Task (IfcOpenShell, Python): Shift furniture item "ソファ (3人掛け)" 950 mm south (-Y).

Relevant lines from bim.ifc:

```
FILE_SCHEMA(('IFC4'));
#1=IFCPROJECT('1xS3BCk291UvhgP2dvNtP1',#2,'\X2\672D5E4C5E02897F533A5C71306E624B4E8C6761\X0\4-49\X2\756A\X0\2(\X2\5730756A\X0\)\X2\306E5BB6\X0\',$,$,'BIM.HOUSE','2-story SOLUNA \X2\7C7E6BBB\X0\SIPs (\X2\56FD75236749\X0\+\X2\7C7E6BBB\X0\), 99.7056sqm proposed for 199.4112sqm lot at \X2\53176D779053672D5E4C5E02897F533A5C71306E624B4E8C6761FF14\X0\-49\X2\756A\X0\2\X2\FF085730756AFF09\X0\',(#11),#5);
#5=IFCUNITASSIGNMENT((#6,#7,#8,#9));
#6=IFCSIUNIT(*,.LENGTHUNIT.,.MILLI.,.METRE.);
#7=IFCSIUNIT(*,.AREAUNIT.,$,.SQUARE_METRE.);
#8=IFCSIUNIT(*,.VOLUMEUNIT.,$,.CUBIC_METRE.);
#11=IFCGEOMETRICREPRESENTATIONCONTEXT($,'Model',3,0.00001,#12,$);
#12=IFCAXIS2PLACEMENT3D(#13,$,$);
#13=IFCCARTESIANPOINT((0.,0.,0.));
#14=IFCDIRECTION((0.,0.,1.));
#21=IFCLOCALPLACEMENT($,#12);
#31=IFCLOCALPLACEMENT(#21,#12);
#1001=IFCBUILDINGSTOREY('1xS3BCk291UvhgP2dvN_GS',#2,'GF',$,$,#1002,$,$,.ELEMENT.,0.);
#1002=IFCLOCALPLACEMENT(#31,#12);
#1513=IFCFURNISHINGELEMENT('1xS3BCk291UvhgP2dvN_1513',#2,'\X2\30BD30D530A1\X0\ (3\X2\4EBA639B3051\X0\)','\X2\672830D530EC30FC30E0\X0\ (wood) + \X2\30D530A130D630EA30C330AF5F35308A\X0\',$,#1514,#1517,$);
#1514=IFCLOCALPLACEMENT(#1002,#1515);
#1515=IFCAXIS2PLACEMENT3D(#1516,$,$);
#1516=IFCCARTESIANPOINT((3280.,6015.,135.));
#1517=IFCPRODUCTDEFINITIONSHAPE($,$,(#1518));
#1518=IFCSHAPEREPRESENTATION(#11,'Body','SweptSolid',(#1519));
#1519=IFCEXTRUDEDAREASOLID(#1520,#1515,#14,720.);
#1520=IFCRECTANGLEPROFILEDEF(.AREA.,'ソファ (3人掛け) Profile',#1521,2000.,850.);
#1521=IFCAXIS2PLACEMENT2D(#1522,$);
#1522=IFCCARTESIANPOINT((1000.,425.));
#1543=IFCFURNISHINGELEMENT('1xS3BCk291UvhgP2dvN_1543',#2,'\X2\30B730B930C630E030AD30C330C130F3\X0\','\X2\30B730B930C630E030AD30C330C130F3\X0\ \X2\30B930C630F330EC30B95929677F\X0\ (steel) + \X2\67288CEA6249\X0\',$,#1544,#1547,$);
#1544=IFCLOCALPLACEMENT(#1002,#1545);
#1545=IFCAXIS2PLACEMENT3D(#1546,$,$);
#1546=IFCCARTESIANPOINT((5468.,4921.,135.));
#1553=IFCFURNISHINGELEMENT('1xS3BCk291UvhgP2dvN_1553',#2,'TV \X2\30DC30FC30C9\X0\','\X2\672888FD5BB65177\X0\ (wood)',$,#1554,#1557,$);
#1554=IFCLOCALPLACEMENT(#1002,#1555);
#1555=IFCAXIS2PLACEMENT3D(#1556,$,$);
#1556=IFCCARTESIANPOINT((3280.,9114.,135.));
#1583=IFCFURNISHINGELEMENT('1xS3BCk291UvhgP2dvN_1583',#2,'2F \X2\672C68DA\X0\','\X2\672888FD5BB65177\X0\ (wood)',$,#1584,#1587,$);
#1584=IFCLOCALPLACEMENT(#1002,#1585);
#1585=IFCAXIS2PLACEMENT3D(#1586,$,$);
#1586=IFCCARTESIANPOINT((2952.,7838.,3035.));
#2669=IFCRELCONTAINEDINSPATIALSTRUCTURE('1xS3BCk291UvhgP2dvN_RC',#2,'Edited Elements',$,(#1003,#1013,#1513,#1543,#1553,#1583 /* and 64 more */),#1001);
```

```python
import ifcopenshell
import ifcopenshell.api.geometry
import ifcopenshell.util.placement
import ifcopenshell.util.unit

model = ifcopenshell.open("bim.ifc")
unit_scale = ifcopenshell.util.unit.calculate_unit_scale(model)

item = model.by_id(1513)
matrix = ifcopenshell.util.placement.get_local_placement(item.ObjectPlacement)
matrix[1, 3] -= 0.95 / unit_scale
ifcopenshell.api.geometry.edit_object_placement(model, product=item, matrix=matrix, is_si=False)

print(ifcopenshell.util.placement.get_local_placement(item.ObjectPlacement).round(3) + 0.0)

model.write("bim_v2.ifc")
```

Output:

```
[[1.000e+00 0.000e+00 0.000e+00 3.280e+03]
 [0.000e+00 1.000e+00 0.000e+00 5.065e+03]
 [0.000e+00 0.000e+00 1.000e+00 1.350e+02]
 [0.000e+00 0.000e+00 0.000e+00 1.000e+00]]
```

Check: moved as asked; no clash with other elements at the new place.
